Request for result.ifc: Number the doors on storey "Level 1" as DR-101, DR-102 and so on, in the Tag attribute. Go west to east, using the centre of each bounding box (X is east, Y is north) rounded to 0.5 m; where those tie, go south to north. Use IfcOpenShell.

First a look at what the model holds.

```python
import ifcopenshell
import ifcopenshell.util.element
import ifcopenshell.util.placement

model = ifcopenshell.open("result.ifc")
print(model.schema)
storey = next(s for s in model.by_type("IfcBuildingStorey") if s.Name == "Level 1")
doors = [e for e in ifcopenshell.util.element.get_decomposition(storey) if e.is_a("IfcDoor")]
for e in sorted(doors, key=lambda e: e.id()):
    origin = ifcopenshell.util.placement.get_local_placement(e.ObjectPlacement)[:3, 3]
    print(e.id(), e.Tag, e.Name, origin.round(2) + 0.0, sep=" | ")
```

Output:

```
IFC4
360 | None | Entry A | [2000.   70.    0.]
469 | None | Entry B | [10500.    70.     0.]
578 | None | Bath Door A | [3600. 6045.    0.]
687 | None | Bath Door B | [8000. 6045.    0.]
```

```python
import ifcopenshell
import ifcopenshell.geom
import ifcopenshell.util.element
import ifcopenshell.util.shape

model = ifcopenshell.open("result.ifc")
settings = ifcopenshell.geom.settings()
settings.set("use-world-coords", True)


def centre(element):
    shape = ifcopenshell.geom.create_shape(settings, element)
    return ifcopenshell.util.shape.get_bbox_centroid(shape.geometry)


storey = next(s for s in model.by_type("IfcBuildingStorey") if s.Name == "Level 1")
doors = [e for e in ifcopenshell.util.element.get_decomposition(storey) if e.is_a("IfcDoor")]

# Insertion points can sit at a corner or the storey origin, so sort by the geometry (in metres).
centres = {e: centre(e) for e in doors}
doors.sort(key=lambda e: (round(centres[e][0] / 0.5), centres[e][1]))

for i, e in enumerate(doors, start=1):
    number = f"DR-1{i:02d}"
    e.Tag = number
    print(e.id(), number)

model.write("result-out.ifc")
```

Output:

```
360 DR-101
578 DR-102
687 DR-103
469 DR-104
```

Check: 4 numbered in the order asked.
